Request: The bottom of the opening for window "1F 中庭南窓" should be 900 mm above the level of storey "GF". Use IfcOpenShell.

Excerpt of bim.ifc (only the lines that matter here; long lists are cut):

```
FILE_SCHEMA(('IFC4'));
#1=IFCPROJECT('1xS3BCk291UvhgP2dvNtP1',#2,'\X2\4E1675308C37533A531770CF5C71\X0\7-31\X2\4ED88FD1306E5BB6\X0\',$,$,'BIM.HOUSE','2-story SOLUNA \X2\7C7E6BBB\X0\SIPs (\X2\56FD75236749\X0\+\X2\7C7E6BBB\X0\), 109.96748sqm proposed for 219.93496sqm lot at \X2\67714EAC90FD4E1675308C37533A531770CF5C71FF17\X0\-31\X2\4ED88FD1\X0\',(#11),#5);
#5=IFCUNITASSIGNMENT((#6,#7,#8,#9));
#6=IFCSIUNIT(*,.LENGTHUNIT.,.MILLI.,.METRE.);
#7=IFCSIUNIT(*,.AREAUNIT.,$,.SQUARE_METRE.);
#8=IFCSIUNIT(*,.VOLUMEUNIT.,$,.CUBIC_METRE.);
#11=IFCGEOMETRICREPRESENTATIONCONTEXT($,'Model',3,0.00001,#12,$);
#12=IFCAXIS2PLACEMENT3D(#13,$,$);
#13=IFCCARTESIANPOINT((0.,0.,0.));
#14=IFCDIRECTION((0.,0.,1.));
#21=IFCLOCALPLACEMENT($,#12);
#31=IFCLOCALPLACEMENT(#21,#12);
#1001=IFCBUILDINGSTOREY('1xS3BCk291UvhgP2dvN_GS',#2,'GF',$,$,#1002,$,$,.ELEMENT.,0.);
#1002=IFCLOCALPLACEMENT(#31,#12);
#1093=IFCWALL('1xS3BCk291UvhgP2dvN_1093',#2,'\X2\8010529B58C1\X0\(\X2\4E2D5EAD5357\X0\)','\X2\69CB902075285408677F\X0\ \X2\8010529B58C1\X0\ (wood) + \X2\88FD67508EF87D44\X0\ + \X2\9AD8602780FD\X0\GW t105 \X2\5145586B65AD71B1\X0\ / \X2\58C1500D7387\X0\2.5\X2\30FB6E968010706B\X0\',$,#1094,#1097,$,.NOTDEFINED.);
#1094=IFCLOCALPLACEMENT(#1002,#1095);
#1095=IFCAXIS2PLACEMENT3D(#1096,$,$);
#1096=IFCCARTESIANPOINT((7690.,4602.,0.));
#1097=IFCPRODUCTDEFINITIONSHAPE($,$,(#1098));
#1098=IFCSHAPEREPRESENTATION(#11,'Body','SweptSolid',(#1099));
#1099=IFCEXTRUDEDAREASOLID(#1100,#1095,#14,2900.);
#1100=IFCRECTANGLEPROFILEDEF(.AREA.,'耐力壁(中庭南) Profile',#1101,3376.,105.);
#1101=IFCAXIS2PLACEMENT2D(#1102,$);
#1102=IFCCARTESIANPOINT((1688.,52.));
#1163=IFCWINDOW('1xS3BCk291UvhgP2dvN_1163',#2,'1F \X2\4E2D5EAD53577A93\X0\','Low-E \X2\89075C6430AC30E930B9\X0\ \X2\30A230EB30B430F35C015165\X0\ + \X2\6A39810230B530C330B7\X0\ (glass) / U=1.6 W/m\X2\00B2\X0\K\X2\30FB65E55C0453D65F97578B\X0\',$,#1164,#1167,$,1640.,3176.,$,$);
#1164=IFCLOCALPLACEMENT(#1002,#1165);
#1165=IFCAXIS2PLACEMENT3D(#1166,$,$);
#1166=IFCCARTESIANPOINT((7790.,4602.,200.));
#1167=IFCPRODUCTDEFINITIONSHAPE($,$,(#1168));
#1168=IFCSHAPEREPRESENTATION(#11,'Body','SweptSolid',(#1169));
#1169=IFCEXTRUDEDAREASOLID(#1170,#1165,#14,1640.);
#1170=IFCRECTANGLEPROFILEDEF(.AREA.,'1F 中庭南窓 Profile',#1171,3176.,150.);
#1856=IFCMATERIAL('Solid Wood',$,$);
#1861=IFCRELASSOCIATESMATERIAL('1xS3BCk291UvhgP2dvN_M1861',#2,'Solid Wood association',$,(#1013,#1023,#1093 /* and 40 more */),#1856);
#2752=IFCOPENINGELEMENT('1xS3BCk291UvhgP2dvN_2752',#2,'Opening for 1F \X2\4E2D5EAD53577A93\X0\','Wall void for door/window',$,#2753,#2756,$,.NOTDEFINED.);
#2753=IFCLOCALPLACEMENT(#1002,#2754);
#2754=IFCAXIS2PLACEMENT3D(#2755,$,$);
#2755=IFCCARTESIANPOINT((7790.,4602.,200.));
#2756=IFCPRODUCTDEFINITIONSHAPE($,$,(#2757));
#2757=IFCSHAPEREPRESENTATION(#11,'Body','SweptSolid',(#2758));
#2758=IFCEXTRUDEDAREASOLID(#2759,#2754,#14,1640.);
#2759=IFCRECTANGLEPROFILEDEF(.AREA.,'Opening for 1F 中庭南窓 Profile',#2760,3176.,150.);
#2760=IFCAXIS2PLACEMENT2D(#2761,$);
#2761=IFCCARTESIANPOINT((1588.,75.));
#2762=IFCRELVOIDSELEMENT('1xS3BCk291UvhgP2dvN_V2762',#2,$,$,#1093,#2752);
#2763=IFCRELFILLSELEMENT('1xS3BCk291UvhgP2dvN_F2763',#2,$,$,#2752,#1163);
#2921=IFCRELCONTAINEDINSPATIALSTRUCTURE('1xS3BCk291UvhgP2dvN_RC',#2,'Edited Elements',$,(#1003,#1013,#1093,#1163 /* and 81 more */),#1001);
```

```python
import numpy as np
import ifcopenshell
import ifcopenshell.api.geometry
import ifcopenshell.geom
import ifcopenshell.util.element
import ifcopenshell.util.placement
import ifcopenshell.util.shape
import ifcopenshell.util.unit

model = ifcopenshell.open("bim.ifc")
unit_scale = ifcopenshell.util.unit.calculate_unit_scale(model)

window = model.by_guid("1xS3BCk291UvhgP2dvN_1163")
opening = window.FillsVoids[0].RelatingOpeningElement
storey = ifcopenshell.util.element.get_container(window, ifc_class="IfcBuildingStorey")
level = ifcopenshell.util.placement.get_local_placement(storey.ObjectPlacement)[2, 3]

# The opening's origin need not be at the sill, so measure its lowest point.
shape = ifcopenshell.geom.create_shape(ifcopenshell.geom.settings(), opening)
bottom = ifcopenshell.util.shape.get_shape_bottom_elevation(shape, shape.geometry) / unit_scale
dz = level + 0.9 / unit_scale - bottom

shift = np.array([0.0, 0.0, dz])
# The window is not placed relative to its opening, so move both.
for product in (opening, window):
    matrix = ifcopenshell.util.placement.get_local_placement(product.ObjectPlacement)
    matrix[:3, 3] += shift
    ifcopenshell.api.geometry.edit_object_placement(model, product=product, matrix=matrix, is_si=False)

print(f"moved by {dz * unit_scale:+.3f} m")

model.write("bim_v2.ifc")
```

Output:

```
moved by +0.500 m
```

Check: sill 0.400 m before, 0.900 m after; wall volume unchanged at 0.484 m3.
